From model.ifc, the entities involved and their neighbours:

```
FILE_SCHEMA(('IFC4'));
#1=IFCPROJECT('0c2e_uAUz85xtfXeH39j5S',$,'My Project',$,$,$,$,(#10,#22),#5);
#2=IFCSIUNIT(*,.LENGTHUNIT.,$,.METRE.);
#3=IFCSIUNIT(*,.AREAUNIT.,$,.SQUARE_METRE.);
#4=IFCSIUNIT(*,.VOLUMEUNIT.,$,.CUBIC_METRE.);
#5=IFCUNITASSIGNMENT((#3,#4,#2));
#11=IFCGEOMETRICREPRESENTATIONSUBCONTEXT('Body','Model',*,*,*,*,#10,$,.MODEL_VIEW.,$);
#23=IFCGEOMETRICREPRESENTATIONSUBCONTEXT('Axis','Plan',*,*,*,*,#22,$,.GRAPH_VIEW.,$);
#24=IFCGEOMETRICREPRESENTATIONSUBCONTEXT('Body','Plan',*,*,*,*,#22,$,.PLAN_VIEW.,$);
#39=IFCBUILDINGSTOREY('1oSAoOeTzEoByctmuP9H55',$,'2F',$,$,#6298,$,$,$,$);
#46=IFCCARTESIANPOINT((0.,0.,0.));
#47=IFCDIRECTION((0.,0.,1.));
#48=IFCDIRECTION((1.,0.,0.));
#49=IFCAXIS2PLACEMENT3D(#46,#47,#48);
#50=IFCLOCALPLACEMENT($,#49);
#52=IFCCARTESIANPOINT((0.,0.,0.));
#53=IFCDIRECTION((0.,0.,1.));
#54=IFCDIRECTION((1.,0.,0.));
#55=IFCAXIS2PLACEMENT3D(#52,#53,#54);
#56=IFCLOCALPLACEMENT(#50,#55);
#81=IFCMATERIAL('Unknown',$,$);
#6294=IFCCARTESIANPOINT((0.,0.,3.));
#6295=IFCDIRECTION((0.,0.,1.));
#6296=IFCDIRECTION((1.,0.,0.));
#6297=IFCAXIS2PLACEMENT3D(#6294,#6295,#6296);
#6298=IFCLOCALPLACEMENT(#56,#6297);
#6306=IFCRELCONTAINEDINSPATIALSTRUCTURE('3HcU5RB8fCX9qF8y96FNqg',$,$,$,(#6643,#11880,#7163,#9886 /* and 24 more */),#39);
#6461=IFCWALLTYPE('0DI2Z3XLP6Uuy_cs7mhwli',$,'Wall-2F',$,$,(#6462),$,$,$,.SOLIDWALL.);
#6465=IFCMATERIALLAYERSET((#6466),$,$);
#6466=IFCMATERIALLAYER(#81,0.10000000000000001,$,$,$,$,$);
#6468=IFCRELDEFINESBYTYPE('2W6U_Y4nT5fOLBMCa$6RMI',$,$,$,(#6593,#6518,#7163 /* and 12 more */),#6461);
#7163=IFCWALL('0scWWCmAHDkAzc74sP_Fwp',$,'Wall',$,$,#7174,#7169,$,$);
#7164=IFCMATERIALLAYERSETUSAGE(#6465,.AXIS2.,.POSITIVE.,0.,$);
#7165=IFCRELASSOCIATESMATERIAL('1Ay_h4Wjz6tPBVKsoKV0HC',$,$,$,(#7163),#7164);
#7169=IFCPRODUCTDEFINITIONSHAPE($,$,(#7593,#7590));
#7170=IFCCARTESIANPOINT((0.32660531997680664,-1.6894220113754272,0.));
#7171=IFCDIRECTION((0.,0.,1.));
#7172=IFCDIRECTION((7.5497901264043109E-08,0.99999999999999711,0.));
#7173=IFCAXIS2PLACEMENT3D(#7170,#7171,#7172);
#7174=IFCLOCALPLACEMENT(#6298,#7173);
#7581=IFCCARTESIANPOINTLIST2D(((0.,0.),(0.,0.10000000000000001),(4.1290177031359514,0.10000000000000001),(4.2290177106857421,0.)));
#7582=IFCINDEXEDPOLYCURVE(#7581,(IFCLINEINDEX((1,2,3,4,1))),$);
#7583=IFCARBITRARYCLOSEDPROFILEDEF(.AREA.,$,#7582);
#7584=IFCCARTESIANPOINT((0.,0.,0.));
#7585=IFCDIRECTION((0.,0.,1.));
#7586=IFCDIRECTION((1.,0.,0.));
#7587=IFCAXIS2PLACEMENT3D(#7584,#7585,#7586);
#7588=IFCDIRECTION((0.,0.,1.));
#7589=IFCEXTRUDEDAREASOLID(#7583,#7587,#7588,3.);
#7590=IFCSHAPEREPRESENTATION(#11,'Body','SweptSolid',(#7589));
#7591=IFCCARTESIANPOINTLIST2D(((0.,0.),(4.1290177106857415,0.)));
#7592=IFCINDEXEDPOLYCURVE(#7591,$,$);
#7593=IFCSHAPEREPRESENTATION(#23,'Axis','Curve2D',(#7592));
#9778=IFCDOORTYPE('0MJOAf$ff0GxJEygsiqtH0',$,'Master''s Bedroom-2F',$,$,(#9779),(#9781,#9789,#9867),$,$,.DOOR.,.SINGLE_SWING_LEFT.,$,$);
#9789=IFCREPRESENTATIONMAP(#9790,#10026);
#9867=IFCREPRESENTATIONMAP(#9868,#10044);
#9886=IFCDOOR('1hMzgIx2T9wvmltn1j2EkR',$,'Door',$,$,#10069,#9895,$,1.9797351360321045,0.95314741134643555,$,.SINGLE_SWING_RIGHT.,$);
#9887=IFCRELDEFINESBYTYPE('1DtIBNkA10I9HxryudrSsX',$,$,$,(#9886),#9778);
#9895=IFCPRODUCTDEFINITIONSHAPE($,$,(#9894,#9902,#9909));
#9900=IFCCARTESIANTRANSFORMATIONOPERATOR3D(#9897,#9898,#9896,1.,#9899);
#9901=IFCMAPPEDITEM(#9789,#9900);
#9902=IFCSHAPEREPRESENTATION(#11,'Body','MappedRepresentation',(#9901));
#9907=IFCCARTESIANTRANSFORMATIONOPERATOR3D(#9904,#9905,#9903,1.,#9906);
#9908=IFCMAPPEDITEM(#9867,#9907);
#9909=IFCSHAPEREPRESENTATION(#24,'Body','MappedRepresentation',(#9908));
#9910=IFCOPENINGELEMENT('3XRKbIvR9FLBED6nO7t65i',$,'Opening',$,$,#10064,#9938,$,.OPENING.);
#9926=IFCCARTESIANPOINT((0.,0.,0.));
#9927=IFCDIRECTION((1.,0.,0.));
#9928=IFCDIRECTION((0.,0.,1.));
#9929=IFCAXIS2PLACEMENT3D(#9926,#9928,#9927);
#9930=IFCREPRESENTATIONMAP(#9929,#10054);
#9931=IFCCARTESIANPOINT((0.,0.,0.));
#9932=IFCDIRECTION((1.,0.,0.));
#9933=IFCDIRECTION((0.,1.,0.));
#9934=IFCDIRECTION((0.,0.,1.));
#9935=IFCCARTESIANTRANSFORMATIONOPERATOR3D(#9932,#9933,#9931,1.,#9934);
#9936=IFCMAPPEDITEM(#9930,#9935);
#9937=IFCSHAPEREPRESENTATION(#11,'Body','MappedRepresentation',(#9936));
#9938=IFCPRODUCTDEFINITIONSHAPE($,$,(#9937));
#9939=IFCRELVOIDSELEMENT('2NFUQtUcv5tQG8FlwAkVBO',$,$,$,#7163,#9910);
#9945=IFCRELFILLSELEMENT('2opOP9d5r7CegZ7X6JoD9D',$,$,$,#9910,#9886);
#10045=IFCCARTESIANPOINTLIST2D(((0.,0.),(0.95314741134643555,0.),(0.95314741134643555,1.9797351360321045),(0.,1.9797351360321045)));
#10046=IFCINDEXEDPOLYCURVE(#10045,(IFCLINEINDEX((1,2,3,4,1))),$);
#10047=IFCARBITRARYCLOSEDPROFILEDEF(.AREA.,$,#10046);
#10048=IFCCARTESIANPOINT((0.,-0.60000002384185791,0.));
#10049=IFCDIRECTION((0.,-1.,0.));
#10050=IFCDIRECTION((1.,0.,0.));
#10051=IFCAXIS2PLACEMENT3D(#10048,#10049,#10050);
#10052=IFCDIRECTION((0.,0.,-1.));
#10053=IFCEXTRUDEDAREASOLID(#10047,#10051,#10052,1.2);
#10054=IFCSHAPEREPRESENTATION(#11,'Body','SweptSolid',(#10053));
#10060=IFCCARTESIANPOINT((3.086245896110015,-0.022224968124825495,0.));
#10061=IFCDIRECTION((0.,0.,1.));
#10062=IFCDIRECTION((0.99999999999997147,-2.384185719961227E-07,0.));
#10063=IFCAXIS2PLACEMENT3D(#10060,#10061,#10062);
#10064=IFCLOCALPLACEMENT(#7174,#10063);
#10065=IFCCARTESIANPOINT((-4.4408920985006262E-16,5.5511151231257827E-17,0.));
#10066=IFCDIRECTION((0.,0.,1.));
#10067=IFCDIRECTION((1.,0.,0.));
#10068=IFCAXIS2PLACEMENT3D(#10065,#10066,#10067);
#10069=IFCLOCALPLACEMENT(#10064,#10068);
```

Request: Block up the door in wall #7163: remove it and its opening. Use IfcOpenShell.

```python
import ifcopenshell
import ifcopenshell.api.feature
import ifcopenshell.api.root
import ifcopenshell.geom
import ifcopenshell.util.shape

model = ifcopenshell.open("model.ifc")
settings = ifcopenshell.geom.settings()


def volume(element):
    """Net volume in cubic metres, openings subtracted."""
    shape = ifcopenshell.geom.create_shape(settings, element)
    return ifcopenshell.util.shape.get_volume(shape.geometry)


door = model.by_guid("1hMzgIx2T9wvmltn1j2EkR")
opening = door.FillsVoids[0].RelatingOpeningElement
wall = opening.VoidsElements[0].RelatingBuildingElement
before = volume(wall)

ifcopenshell.api.root.remove_product(model, product=door)
ifcopenshell.api.feature.remove_feature(model, feature=opening)

after = volume(wall)

print(f"wall volume {before:.3f} -> {after:.3f} m3")

model.write("model_rev.ifc")
```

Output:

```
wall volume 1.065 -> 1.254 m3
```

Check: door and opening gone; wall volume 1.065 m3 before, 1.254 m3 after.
